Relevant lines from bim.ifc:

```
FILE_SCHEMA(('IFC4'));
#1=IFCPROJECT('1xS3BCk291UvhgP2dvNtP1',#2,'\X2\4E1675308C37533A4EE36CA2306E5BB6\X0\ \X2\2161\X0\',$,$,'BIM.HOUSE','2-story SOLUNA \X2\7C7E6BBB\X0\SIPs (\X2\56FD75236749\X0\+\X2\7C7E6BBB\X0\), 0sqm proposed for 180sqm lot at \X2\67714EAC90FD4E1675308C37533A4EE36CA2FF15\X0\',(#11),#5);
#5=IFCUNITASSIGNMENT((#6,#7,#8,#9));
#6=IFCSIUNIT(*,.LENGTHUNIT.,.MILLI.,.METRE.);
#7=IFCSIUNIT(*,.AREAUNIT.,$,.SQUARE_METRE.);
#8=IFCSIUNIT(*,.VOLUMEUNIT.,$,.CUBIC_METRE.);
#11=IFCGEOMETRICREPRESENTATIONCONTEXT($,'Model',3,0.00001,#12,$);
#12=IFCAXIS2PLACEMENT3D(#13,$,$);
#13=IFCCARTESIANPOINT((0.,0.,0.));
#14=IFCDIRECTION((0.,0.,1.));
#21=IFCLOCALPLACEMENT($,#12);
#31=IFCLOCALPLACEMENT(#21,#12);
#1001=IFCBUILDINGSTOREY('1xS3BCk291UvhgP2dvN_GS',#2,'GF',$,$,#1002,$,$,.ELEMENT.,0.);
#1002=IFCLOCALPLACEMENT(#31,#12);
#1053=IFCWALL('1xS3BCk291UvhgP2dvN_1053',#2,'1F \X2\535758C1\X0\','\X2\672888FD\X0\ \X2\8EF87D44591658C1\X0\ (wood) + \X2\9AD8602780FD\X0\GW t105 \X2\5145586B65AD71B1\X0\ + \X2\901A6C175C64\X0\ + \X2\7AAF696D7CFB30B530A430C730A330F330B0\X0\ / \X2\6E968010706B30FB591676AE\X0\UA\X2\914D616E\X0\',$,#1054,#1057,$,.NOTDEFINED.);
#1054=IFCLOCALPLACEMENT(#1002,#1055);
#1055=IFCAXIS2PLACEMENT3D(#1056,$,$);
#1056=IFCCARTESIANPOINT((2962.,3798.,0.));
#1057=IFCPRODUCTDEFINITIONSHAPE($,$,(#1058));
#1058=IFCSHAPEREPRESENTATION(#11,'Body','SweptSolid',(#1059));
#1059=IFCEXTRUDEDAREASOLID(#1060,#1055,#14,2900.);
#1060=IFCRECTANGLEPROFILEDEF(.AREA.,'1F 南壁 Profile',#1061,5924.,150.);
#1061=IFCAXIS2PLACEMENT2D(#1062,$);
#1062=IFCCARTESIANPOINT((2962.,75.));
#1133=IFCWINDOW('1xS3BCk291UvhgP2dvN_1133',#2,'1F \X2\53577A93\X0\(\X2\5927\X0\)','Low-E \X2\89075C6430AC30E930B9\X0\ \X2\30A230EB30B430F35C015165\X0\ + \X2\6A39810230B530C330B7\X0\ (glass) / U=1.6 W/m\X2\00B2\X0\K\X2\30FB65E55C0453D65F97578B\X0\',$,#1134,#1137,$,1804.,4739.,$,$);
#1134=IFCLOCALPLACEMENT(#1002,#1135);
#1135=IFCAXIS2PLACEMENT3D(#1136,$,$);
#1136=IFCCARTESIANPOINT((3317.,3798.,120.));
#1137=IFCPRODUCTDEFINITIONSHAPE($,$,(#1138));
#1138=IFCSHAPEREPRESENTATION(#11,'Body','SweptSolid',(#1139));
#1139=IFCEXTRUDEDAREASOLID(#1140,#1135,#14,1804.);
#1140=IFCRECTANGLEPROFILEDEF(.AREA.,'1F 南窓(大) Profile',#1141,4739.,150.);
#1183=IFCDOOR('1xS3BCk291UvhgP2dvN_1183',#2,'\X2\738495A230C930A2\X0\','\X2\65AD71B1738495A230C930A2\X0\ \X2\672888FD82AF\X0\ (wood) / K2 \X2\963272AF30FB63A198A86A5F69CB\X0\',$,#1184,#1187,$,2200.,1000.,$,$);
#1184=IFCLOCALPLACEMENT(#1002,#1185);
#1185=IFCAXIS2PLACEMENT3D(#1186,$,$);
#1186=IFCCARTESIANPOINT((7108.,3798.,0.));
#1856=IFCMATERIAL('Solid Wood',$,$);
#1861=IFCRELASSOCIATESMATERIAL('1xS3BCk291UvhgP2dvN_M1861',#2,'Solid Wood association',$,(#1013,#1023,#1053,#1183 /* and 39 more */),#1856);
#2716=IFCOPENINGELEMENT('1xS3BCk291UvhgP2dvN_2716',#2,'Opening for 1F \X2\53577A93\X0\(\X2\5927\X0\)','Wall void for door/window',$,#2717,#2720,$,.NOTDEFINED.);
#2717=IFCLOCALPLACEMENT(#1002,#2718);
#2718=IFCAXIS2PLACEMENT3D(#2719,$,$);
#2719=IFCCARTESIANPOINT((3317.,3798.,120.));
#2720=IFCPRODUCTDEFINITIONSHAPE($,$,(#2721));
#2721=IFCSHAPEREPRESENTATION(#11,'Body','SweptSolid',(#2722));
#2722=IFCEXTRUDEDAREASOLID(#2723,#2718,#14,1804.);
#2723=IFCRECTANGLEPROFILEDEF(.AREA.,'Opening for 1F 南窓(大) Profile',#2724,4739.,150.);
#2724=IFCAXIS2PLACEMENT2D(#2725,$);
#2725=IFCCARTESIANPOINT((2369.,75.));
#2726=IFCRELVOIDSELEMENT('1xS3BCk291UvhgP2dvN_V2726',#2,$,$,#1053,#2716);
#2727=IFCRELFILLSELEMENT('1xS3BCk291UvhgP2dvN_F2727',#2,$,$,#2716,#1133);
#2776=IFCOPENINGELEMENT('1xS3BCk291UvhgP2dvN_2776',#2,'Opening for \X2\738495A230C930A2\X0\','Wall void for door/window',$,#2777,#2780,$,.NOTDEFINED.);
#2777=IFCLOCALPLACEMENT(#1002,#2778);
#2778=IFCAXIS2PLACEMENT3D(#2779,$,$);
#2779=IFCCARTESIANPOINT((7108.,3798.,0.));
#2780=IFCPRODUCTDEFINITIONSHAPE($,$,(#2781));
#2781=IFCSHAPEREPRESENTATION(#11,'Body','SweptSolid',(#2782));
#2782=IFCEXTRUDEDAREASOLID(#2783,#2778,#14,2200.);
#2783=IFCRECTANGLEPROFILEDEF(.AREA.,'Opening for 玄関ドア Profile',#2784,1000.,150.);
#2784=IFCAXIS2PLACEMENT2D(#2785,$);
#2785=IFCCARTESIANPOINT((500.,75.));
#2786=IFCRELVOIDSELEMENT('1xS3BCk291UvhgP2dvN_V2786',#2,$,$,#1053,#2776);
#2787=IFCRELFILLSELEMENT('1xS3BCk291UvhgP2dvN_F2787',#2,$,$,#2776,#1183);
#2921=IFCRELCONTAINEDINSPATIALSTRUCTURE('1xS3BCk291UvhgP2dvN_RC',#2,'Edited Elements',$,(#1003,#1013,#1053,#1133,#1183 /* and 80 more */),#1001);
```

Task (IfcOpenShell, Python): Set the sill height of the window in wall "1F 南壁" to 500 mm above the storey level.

```python
import numpy as np
import ifcopenshell
import ifcopenshell.api.geometry
import ifcopenshell.geom
import ifcopenshell.util.element
import ifcopenshell.util.placement
import ifcopenshell.util.shape
import ifcopenshell.util.unit

model = ifcopenshell.open("bim.ifc")
unit_scale = ifcopenshell.util.unit.calculate_unit_scale(model)

window = model.by_id(1133)
opening = window.FillsVoids[0].RelatingOpeningElement
storey = ifcopenshell.util.element.get_container(window, ifc_class="IfcBuildingStorey")
level = ifcopenshell.util.placement.get_local_placement(storey.ObjectPlacement)[2, 3]

# The opening's origin need not be at the sill, so measure its lowest point.
shape = ifcopenshell.geom.create_shape(ifcopenshell.geom.settings(), opening)
bottom = ifcopenshell.util.shape.get_shape_bottom_elevation(shape, shape.geometry) / unit_scale
dz = level + 500.0 - bottom

shift = np.array([0.0, 0.0, dz])
# The window is not placed relative to its opening, so move both.
for product in (opening, window):
    matrix = ifcopenshell.util.placement.get_local_placement(product.ObjectPlacement)
    matrix[:3, 3] += shift
    ifcopenshell.api.geometry.edit_object_placement(model, product=product, matrix=matrix, is_si=False)

print(f"moved by {dz * unit_scale:+.3f} m")

model.write("bim_v2.ifc")
```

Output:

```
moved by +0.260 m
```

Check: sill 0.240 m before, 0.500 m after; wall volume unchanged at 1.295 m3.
